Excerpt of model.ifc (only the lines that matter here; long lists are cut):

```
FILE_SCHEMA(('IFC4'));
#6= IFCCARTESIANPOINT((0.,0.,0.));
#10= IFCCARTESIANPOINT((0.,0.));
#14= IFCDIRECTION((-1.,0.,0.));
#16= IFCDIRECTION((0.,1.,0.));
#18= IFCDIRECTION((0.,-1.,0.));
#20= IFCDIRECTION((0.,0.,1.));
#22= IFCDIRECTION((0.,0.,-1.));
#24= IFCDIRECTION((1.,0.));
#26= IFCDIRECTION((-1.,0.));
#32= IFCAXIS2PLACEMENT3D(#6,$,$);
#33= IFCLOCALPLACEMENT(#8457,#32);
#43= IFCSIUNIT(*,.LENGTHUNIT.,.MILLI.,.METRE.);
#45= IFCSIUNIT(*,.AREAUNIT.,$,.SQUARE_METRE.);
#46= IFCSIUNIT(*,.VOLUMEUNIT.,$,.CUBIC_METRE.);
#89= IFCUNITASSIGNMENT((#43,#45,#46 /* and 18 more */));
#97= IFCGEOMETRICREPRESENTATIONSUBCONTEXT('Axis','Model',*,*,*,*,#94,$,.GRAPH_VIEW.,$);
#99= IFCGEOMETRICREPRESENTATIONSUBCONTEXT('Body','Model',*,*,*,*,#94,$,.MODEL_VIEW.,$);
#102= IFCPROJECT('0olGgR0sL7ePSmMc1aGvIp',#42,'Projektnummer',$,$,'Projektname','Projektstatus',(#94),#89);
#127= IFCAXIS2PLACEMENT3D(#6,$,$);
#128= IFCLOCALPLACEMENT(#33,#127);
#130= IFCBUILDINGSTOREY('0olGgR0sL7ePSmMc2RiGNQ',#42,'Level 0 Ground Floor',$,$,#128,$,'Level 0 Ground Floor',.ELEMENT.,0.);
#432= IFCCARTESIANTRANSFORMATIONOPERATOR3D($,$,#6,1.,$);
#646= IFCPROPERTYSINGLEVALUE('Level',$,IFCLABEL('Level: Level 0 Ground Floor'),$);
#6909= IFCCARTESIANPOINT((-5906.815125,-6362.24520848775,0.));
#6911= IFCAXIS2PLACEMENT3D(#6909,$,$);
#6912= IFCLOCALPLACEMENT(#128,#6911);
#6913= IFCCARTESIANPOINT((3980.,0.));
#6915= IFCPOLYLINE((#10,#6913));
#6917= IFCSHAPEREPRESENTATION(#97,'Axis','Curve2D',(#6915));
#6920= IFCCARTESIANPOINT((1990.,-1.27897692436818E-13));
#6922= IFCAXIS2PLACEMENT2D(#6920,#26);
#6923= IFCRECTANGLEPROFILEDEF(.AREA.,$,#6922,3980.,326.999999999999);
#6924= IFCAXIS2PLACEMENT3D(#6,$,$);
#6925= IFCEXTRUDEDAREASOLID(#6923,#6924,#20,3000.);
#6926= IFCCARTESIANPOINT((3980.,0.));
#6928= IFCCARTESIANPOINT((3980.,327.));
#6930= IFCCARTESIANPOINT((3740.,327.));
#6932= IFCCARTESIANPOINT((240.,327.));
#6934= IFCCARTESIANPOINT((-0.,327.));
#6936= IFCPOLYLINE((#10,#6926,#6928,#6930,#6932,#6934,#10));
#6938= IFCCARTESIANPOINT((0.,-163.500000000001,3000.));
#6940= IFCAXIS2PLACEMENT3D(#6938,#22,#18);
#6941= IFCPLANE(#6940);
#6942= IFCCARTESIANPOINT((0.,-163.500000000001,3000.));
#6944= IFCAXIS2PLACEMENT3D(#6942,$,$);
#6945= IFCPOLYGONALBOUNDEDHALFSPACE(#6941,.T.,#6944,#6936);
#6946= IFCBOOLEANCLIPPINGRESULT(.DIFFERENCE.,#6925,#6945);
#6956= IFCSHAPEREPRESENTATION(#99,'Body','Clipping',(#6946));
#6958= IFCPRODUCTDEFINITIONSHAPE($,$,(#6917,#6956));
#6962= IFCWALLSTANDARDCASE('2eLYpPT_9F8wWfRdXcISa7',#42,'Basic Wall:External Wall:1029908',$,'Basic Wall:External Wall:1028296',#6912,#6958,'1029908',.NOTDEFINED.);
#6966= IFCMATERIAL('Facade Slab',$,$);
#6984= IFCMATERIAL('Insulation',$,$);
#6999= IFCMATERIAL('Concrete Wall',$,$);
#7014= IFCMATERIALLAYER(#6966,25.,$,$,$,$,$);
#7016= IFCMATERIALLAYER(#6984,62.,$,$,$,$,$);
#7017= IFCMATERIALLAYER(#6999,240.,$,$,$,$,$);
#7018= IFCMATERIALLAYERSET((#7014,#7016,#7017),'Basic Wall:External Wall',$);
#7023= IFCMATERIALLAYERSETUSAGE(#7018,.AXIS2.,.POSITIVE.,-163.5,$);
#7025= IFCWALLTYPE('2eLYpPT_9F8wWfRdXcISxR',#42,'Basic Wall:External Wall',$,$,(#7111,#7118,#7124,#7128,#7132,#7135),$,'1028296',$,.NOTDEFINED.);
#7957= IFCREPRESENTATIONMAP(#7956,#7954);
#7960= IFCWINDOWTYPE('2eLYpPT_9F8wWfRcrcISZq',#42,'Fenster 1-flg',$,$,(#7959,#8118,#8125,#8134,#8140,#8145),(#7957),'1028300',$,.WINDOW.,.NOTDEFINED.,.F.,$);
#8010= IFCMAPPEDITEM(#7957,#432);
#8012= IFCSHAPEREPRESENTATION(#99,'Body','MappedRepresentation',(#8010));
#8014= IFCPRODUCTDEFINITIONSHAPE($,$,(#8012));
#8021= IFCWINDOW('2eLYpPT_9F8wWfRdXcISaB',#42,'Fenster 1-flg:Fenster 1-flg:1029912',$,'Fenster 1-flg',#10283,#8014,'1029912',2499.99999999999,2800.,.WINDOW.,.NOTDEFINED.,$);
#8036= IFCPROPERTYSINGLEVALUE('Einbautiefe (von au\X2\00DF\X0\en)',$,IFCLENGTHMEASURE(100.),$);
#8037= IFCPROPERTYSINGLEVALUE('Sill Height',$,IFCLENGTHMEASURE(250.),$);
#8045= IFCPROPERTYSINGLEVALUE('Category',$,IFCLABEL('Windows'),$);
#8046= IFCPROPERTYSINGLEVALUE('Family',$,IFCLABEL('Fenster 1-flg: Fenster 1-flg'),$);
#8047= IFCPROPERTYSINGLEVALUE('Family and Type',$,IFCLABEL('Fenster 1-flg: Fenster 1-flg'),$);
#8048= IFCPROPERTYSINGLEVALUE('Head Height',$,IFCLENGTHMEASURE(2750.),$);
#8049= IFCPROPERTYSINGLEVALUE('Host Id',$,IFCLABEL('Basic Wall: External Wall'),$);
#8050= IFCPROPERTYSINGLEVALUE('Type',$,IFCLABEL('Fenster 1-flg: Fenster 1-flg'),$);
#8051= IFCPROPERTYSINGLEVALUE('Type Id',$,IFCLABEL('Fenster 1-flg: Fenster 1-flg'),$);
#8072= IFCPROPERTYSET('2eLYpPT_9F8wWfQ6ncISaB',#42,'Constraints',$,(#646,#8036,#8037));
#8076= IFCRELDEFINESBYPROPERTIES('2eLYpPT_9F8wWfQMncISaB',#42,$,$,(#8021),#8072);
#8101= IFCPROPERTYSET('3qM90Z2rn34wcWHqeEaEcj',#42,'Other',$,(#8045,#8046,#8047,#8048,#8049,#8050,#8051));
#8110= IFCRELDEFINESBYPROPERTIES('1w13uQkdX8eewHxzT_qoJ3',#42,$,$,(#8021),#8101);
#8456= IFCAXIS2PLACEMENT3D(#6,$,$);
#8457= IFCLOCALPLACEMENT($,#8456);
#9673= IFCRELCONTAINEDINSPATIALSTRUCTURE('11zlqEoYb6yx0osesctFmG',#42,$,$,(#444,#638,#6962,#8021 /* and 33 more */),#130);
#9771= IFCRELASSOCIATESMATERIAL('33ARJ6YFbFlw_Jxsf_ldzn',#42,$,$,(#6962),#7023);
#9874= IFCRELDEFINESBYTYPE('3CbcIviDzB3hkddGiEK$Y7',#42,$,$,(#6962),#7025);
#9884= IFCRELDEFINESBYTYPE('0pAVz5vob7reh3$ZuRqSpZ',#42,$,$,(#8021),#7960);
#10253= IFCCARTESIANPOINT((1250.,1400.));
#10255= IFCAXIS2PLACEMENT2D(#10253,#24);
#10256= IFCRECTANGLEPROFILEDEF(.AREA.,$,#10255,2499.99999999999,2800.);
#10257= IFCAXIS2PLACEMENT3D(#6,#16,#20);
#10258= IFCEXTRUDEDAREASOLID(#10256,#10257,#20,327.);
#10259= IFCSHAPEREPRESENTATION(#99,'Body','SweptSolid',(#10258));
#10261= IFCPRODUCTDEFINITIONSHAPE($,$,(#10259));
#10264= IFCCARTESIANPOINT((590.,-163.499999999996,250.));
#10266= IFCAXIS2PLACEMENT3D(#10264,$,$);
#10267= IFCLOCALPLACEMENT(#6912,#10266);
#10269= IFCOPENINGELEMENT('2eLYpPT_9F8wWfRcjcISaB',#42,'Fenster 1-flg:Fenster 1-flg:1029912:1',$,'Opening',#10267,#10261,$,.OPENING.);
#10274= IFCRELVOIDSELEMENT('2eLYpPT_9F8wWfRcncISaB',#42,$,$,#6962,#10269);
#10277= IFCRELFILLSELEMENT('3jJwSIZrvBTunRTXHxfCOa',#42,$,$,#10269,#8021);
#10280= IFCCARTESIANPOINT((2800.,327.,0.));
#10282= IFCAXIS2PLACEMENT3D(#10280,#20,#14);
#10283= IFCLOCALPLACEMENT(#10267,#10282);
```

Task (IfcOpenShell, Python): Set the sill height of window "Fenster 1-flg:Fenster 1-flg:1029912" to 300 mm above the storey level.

```python
import numpy as np
import ifcopenshell
import ifcopenshell.api.geometry
import ifcopenshell.api.pset
import ifcopenshell.geom
import ifcopenshell.util.element
import ifcopenshell.util.placement
import ifcopenshell.util.shape
import ifcopenshell.util.unit

model = ifcopenshell.open("model.ifc")
unit_scale = ifcopenshell.util.unit.calculate_unit_scale(model)

window = model.by_guid("2eLYpPT_9F8wWfRdXcISaB")
opening = window.FillsVoids[0].RelatingOpeningElement
storey = ifcopenshell.util.element.get_container(window, ifc_class="IfcBuildingStorey")
level = ifcopenshell.util.placement.get_local_placement(storey.ObjectPlacement)[2, 3]

# The opening's origin need not be at the sill, so measure its lowest point.
shape = ifcopenshell.geom.create_shape(ifcopenshell.geom.settings(), opening)
bottom = ifcopenshell.util.shape.get_shape_bottom_elevation(shape, shape.geometry) / unit_scale
dz = level + 0.3 / unit_scale - bottom

shift = np.array([0.0, 0.0, dz])
# The window is placed relative to its opening, so it follows when the opening moves.
matrix = ifcopenshell.util.placement.get_local_placement(opening.ObjectPlacement)
matrix[:3, 3] += shift
ifcopenshell.api.geometry.edit_object_placement(
    model, product=opening, matrix=matrix, is_si=False, should_transform_children=True
)

# Keep the stored heights in step.
pset = model.by_id(ifcopenshell.util.element.get_pset(window, "Constraints", should_inherit=False)["id"])
ifcopenshell.api.pset.edit_pset(model, pset=pset, properties={
    "Sill Height": model.create_entity("IfcLengthMeasure", ifcopenshell.util.element.get_pset(window, "Constraints", "Sill Height") + dz),
})
pset = model.by_id(ifcopenshell.util.element.get_pset(window, "Other", should_inherit=False)["id"])
ifcopenshell.api.pset.edit_pset(model, pset=pset, properties={
    "Head Height": model.create_entity("IfcLengthMeasure", ifcopenshell.util.element.get_pset(window, "Other", "Head Height") + dz),
})

print(f"moved by {dz * unit_scale:+.3f} m")

model.write("model_updated.ifc")
```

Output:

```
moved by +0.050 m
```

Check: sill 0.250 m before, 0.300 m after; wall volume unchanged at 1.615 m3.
